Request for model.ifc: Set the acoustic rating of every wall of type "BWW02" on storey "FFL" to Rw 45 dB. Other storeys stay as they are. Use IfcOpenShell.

First a look at what the model holds.

```python
import ifcopenshell
import ifcopenshell.util.element

model = ifcopenshell.open("model.ifc")
print(model.schema)
storey = next(s for s in model.by_type("IfcBuildingStorey") if s.Name == "FFL")
walls = [e for e in ifcopenshell.util.element.get_decomposition(storey) if e.is_a("IfcWall")]
seen = {}
for e in walls:
    element_type = ifcopenshell.util.element.get_type(e)
    key = (element_type.Name if element_type != e and element_type else None, ifcopenshell.util.element.get_pset(e, "Pset_WallCommon", "AcousticRating"))
    seen[key] = seen.get(key, 0) + 1
for (name, value), count in sorted(seen.items(), key=str):
    print(count, "x", name, "|", value)
```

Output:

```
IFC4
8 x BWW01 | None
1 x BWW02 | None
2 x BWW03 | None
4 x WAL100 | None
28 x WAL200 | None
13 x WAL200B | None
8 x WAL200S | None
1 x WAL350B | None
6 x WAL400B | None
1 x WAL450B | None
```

```python
import ifcopenshell
import ifcopenshell.api.pset
import ifcopenshell.util.element

model = ifcopenshell.open("model.ifc")

storey = next(s for s in model.by_type("IfcBuildingStorey") if s.Name == "FFL")
walls = [e for e in ifcopenshell.util.element.get_decomposition(storey) if e.is_a("IfcWall")]

count = 0
for e in walls:
    element_type = ifcopenshell.util.element.get_type(e)
    if element_type in (None, e) or element_type.Name != "BWW02":
        continue
    # add_pset returns the element's existing set when there is one.
    pset = ifcopenshell.api.pset.add_pset(model, product=e, name="Pset_WallCommon")
    ifcopenshell.api.pset.edit_pset(model, pset=pset, properties={"AcousticRating": "Rw 45 dB"})
    count += 1

print(count, "walls updated")

model.write("model_updated.ifc")
```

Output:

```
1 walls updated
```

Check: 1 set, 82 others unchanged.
